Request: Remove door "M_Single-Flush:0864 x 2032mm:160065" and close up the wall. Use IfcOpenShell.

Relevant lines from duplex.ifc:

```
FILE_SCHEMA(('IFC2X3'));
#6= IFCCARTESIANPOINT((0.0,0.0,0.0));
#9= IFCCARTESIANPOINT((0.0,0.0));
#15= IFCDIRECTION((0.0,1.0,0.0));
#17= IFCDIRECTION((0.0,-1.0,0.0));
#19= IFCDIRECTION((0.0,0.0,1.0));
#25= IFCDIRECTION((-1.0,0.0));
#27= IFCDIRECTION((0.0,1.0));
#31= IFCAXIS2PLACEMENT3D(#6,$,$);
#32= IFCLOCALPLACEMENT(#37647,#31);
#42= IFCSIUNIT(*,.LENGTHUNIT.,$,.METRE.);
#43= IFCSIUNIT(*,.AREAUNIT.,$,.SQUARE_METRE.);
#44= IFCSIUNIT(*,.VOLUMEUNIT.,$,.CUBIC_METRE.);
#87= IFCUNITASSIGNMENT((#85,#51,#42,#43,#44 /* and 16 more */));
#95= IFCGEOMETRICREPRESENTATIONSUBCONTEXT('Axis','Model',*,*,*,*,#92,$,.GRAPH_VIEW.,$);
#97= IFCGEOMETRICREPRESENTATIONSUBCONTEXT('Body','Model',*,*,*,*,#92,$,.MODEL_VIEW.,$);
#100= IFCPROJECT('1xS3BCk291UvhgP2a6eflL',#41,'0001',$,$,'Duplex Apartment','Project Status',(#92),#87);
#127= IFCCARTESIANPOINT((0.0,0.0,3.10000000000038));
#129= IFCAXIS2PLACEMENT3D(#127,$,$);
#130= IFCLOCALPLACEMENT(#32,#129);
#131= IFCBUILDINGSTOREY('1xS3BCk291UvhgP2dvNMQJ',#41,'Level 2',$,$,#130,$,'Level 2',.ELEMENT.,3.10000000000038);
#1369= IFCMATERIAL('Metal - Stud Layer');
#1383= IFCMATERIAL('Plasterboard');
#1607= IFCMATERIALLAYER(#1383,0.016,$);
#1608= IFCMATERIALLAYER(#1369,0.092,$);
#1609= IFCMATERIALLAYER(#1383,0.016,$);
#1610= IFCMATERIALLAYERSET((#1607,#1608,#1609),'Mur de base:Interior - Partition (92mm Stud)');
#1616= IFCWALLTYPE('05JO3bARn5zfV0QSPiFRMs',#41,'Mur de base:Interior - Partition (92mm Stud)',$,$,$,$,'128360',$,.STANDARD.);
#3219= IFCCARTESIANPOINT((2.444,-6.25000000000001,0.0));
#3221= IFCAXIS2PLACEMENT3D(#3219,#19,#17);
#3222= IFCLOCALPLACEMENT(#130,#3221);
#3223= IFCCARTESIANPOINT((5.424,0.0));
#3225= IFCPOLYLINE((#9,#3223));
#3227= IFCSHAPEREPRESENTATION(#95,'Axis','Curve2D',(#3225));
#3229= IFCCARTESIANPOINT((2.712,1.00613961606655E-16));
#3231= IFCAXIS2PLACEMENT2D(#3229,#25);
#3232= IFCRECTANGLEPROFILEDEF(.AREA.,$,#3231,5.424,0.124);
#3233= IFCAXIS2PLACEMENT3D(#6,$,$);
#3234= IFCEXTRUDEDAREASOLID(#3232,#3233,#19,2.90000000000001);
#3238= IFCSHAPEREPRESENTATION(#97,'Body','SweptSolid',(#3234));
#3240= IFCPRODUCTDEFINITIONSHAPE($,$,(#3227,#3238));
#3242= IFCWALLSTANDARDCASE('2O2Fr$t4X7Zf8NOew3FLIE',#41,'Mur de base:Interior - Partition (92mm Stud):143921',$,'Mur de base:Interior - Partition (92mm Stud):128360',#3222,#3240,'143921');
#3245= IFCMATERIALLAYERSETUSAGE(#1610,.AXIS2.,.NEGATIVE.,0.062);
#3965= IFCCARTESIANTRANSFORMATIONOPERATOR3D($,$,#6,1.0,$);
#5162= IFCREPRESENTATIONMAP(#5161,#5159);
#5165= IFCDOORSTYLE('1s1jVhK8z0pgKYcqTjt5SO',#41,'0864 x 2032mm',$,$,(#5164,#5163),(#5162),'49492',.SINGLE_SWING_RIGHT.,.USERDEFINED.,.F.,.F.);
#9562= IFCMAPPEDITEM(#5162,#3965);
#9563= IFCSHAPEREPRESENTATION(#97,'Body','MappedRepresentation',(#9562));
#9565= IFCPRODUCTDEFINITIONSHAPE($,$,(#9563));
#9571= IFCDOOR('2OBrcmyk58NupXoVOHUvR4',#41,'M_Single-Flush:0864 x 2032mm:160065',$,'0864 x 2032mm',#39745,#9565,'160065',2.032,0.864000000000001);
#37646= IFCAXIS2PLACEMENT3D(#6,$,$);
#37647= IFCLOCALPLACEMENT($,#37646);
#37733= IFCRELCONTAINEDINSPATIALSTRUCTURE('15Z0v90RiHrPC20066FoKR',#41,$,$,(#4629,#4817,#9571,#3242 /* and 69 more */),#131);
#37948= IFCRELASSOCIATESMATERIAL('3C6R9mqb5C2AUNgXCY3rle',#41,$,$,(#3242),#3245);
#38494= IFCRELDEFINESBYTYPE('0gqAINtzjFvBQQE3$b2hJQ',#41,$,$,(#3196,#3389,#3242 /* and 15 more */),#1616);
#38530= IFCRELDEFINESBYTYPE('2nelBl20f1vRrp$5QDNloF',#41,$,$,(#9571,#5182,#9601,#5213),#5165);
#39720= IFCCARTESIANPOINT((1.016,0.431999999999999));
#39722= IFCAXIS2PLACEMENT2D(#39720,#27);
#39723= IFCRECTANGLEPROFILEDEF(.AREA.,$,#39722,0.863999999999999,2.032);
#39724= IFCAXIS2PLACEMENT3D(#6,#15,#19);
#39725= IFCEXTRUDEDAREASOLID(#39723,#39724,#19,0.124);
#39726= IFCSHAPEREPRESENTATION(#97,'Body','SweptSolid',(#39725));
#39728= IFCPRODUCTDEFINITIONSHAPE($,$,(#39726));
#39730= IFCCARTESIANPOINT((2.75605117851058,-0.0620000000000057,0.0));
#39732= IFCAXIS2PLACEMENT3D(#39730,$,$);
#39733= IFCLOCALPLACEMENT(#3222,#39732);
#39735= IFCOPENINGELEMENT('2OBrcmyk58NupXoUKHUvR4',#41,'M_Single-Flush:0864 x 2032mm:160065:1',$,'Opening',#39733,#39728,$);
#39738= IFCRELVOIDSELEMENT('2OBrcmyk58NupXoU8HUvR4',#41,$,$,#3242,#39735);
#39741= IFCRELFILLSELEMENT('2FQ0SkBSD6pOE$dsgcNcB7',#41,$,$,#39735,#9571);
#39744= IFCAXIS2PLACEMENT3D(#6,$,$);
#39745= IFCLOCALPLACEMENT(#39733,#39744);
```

```python
import ifcopenshell
import ifcopenshell.api.feature
import ifcopenshell.api.root
import ifcopenshell.geom
import ifcopenshell.util.shape

model = ifcopenshell.open("duplex.ifc")
settings = ifcopenshell.geom.settings()


def volume(element):
    """Net volume in cubic metres, openings subtracted."""
    shape = ifcopenshell.geom.create_shape(settings, element)
    return ifcopenshell.util.shape.get_volume(shape.geometry)


door = model.by_guid("2OBrcmyk58NupXoVOHUvR4")
opening = door.FillsVoids[0].RelatingOpeningElement
wall = opening.VoidsElements[0].RelatingBuildingElement
before = volume(wall)

ifcopenshell.api.root.remove_product(model, product=door)
ifcopenshell.api.feature.remove_feature(model, feature=opening)

after = volume(wall)

print(f"wall volume {before:.3f} -> {after:.3f} m3")

model.write("duplex-out.ifc")
```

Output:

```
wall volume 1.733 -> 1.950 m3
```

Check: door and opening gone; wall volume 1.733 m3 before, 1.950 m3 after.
